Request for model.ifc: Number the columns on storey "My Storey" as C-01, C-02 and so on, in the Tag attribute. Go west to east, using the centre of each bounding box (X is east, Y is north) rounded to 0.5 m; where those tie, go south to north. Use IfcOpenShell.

First a look at what the model holds.

```python
import ifcopenshell
import ifcopenshell.util.element
import ifcopenshell.util.placement

model = ifcopenshell.open("model.ifc")
print(model.schema)
storey = next(s for s in model.by_type("IfcBuildingStorey") if s.Name == "My Storey")
columns = [e for e in ifcopenshell.util.element.get_decomposition(storey) if e.is_a("IfcColumn")]
for e in sorted(columns, key=lambda e: e.id()):
    origin = ifcopenshell.util.placement.get_local_placement(e.ObjectPlacement)[:3, 3]
    print(e.id(), e.Tag, e.Name, origin.round(2) + 0.0, sep=" | ")
```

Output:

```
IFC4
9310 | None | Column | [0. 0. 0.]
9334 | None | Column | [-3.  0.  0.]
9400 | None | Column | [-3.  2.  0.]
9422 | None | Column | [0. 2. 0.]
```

```python
import ifcopenshell
import ifcopenshell.geom
import ifcopenshell.util.element
import ifcopenshell.util.shape

model = ifcopenshell.open("model.ifc")
settings = ifcopenshell.geom.settings()
settings.set("use-world-coords", True)


def centre(element):
    shape = ifcopenshell.geom.create_shape(settings, element)
    return ifcopenshell.util.shape.get_bbox_centroid(shape.geometry)


storey = next(s for s in model.by_type("IfcBuildingStorey") if s.Name == "My Storey")
columns = [e for e in ifcopenshell.util.element.get_decomposition(storey) if e.is_a("IfcColumn")]

# Insertion points can sit at a corner or the storey origin, so sort by the geometry (in metres).
centres = {e: centre(e) for e in columns}
columns.sort(key=lambda e: (round(centres[e][0] / 0.5), centres[e][1]))

for i, e in enumerate(columns, start=1):
    number = f"C-{i:02d}"
    e.Tag = number
    print(e.id(), number)

model.write("model_edited.ifc")
```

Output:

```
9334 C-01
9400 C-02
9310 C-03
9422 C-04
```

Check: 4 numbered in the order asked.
